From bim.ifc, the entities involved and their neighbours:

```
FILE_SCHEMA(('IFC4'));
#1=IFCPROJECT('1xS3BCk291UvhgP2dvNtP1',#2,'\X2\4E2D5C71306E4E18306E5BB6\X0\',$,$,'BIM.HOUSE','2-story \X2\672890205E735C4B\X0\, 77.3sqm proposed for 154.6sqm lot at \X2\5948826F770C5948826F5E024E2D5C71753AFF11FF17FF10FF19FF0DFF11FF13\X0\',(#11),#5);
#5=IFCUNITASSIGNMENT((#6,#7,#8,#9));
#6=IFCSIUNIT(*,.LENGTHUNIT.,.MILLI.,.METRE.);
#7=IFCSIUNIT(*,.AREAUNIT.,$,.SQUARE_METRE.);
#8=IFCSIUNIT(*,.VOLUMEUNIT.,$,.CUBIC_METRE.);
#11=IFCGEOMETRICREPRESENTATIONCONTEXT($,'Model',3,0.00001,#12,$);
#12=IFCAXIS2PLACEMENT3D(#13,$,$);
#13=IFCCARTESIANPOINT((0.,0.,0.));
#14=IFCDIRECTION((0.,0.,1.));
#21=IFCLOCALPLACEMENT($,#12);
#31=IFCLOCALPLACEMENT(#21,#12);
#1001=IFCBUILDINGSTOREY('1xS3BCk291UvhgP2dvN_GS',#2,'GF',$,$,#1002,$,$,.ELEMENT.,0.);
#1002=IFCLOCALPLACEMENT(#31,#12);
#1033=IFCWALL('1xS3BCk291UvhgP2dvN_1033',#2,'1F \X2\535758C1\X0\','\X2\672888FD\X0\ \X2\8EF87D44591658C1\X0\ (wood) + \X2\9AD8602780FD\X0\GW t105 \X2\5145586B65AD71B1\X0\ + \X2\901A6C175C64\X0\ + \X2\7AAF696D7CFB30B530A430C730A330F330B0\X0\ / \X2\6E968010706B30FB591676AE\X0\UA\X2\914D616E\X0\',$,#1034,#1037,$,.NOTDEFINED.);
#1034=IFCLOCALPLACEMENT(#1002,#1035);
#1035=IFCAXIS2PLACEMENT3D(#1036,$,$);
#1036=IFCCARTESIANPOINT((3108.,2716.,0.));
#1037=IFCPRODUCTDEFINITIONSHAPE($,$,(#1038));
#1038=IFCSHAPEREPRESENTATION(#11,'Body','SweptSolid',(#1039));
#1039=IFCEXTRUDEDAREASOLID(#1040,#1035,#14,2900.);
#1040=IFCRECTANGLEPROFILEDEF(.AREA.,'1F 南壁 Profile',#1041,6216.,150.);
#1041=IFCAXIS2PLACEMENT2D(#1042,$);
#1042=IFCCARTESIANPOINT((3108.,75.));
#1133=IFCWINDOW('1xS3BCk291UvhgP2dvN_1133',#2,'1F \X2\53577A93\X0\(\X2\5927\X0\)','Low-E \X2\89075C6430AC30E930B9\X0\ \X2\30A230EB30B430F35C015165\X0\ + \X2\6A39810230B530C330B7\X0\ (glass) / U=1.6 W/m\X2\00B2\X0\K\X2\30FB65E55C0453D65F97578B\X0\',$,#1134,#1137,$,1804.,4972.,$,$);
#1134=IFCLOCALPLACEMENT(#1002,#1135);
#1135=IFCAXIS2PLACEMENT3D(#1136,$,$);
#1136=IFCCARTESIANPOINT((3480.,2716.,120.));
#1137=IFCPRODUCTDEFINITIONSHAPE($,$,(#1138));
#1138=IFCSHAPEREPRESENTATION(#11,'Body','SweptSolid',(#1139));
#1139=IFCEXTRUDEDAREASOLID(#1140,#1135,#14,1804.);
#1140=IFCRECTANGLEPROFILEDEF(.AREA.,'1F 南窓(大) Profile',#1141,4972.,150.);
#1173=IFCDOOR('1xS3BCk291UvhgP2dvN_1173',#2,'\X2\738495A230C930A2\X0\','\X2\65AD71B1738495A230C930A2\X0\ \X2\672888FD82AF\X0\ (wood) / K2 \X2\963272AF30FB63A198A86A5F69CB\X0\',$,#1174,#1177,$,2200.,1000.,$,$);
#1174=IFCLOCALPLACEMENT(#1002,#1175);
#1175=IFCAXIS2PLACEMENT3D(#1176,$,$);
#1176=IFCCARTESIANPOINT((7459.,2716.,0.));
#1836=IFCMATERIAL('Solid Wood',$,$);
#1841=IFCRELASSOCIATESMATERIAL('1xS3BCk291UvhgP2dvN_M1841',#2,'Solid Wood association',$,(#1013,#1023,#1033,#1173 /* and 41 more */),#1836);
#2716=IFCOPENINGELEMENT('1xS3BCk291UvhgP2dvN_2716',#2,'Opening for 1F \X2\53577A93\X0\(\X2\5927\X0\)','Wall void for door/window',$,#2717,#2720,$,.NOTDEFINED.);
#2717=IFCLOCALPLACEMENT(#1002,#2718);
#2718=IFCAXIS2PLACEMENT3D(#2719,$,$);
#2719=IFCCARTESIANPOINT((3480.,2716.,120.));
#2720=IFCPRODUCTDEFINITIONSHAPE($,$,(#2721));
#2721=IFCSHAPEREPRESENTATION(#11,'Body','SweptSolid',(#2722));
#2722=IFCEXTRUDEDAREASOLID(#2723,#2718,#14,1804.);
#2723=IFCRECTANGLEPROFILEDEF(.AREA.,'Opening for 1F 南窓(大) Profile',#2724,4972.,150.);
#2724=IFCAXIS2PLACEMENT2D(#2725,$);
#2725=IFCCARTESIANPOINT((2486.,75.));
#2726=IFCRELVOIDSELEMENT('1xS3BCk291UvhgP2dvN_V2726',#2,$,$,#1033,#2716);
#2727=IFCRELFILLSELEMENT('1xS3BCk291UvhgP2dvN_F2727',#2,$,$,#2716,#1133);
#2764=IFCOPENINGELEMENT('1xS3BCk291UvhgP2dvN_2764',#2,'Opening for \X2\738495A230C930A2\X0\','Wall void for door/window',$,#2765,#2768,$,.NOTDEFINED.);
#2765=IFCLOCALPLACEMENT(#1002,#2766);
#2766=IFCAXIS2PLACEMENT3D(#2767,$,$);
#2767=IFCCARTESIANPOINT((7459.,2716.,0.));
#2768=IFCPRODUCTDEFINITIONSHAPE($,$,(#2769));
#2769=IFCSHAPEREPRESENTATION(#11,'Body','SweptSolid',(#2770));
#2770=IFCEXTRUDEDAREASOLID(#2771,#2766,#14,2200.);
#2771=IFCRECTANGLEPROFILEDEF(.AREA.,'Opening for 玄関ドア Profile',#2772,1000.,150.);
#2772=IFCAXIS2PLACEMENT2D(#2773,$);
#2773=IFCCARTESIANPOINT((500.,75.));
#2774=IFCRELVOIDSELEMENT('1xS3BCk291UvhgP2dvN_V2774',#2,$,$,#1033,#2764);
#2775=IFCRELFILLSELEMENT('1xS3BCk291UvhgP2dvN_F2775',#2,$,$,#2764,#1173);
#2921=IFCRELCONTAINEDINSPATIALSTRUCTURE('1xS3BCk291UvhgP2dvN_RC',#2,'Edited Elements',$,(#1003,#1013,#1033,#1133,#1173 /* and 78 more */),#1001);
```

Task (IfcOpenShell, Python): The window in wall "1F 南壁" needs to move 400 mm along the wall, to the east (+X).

```python
import ifcopenshell
import ifcopenshell.api.geometry
import ifcopenshell.util.placement

model = ifcopenshell.open("bim.ifc")

window = model.by_id(1133)
opening = window.FillsVoids[0].RelatingOpeningElement
wall = opening.VoidsElements[0].RelatingBuildingElement

wall_matrix = ifcopenshell.util.placement.get_local_placement(wall.ObjectPlacement)
shift = wall_matrix[:3, 0] * 400.0
before = ifcopenshell.util.placement.get_local_placement(window.ObjectPlacement)[:3, 3].copy()

# The window is not placed relative to its opening, so move both.
for product in (opening, window):
    matrix = ifcopenshell.util.placement.get_local_placement(product.ObjectPlacement)
    matrix[:3, 3] += shift
    ifcopenshell.api.geometry.edit_object_placement(model, product=product, matrix=matrix, is_si=False)

after = ifcopenshell.util.placement.get_local_placement(window.ObjectPlacement)[:3, 3]
print("window moved by", (after - before).round(3) + 0.0)

model.write("bim-out.ifc")
```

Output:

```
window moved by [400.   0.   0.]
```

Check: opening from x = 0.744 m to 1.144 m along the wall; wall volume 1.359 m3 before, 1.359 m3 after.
